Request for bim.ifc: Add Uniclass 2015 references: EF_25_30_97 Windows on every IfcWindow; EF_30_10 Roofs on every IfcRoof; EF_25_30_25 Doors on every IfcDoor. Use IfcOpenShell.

First a look at what the model holds.

```python
import ifcopenshell

model = ifcopenshell.open("bim.ifc")
print(model.schema)
print("classifications:", [c.Name for c in model.by_type("IfcClassification")])
for ifc_class in ("IfcDoor", "IfcRoof", "IfcStair", "IfcWall", "IfcWindow"):
    print(ifc_class, len(model.by_type(ifc_class)))
```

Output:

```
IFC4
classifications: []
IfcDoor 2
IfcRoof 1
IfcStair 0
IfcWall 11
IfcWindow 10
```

```python
import ifcopenshell
import ifcopenshell.api.classification

model = ifcopenshell.open("bim.ifc")

system = ifcopenshell.api.classification.add_classification(model, classification="Uniclass 2015")

codes = {
    "IfcWindow": ("EF_25_30_97", "Windows"),
    "IfcRoof": ("EF_30_10", "Roofs"),
    "IfcDoor": ("EF_25_30_25", "Doors"),
}
for ifc_class, (code, name) in codes.items():
    products = model.by_type(ifc_class)
    ifcopenshell.api.classification.add_reference(
        model, products=products, classification=system, identification=code, name=name
    )
    print(code, len(products))

model.write("bim_rev.ifc")
```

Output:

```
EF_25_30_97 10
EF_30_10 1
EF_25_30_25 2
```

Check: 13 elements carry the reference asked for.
